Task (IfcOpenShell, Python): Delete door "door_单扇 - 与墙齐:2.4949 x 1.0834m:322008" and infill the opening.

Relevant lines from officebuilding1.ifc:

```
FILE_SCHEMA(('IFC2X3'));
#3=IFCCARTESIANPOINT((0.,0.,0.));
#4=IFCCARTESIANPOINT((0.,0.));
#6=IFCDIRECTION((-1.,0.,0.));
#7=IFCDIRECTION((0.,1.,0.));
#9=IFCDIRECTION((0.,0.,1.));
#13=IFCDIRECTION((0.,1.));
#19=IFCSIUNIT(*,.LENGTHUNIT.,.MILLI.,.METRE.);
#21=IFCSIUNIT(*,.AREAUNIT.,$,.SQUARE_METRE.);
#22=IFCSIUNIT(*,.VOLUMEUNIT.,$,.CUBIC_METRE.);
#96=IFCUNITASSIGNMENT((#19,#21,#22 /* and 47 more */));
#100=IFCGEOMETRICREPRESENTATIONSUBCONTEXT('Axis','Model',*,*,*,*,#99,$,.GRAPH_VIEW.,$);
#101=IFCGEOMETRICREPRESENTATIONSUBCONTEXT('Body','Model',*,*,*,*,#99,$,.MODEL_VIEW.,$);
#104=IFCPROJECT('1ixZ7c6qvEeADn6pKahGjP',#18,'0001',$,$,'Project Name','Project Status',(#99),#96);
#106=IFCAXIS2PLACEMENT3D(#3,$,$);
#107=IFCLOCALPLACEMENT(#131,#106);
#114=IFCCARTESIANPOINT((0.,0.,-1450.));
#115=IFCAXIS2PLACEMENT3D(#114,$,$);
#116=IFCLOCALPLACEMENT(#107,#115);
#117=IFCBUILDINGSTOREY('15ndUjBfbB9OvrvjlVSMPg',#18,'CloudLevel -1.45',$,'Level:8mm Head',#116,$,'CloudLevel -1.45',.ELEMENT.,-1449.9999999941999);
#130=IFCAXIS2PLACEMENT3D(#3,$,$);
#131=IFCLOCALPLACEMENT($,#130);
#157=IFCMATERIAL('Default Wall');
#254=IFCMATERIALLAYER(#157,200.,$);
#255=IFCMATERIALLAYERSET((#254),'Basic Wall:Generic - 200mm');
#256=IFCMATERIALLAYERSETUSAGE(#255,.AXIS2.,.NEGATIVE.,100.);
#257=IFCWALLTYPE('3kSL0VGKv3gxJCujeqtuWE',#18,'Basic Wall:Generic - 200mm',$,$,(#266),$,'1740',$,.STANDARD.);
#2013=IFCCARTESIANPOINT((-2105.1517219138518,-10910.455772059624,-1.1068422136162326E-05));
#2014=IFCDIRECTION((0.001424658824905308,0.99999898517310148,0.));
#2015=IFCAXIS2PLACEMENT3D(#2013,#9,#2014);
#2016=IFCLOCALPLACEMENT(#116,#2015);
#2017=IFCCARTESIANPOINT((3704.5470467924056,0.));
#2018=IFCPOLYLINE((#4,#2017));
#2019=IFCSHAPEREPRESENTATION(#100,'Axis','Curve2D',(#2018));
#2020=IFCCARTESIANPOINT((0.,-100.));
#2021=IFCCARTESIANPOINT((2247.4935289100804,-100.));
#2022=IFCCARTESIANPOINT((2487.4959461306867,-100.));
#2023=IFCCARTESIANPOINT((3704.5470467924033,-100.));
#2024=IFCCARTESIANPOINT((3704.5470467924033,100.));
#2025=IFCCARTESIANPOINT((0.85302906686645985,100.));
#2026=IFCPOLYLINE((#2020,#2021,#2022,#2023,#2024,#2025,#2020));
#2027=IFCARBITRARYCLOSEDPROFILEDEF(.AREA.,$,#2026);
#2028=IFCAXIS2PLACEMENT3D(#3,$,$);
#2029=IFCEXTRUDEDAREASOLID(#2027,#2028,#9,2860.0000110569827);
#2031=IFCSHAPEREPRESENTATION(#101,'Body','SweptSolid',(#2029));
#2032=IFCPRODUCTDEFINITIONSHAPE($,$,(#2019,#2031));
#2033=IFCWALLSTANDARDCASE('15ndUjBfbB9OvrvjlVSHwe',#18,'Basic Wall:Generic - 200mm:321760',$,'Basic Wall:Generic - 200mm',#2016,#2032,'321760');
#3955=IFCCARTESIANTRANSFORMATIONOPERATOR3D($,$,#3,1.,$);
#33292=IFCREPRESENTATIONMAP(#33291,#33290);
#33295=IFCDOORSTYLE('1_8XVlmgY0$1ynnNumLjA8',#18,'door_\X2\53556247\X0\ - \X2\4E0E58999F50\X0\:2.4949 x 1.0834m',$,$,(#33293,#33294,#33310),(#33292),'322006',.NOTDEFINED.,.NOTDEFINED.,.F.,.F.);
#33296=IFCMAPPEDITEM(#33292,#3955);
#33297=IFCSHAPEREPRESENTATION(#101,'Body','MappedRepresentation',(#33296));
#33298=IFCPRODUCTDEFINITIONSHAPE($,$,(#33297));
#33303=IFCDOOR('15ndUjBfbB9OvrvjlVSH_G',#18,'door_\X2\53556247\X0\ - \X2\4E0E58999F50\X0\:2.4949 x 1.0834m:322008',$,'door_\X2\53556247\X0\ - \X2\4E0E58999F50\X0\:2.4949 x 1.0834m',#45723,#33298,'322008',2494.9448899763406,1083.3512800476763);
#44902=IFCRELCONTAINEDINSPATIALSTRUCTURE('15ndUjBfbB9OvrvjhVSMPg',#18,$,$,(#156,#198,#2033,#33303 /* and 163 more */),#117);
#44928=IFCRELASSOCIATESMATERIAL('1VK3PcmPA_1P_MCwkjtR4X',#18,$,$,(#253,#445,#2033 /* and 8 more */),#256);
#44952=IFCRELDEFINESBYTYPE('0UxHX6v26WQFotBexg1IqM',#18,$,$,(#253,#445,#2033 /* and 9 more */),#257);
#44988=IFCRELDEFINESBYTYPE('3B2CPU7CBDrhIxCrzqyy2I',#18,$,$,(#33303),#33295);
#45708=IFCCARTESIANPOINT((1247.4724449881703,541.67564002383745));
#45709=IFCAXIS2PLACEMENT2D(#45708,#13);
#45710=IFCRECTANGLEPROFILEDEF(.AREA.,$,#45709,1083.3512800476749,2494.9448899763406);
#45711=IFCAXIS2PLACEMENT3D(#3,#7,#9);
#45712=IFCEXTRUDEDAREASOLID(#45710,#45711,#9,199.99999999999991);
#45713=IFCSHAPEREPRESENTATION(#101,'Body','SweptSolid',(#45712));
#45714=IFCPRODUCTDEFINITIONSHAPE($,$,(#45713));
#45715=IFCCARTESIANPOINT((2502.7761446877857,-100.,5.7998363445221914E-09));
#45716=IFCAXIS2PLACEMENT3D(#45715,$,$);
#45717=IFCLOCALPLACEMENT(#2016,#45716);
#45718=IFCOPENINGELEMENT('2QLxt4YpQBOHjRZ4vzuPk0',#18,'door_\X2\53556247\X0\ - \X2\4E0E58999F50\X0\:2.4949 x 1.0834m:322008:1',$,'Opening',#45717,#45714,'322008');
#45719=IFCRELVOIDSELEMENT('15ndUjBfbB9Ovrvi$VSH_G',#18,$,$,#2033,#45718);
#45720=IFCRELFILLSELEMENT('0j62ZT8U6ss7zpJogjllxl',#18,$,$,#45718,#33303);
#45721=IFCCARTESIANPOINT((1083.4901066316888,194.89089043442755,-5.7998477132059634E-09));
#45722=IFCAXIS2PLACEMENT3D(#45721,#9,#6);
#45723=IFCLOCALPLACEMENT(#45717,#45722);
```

```python
import ifcopenshell
import ifcopenshell.api.feature
import ifcopenshell.api.root
import ifcopenshell.geom
import ifcopenshell.util.shape

model = ifcopenshell.open("officebuilding1.ifc")
settings = ifcopenshell.geom.settings()


def volume(element):
    """Net volume in cubic metres, openings subtracted."""
    shape = ifcopenshell.geom.create_shape(settings, element)
    return ifcopenshell.util.shape.get_volume(shape.geometry)


door = model.by_guid("15ndUjBfbB9OvrvjlVSH_G")
opening = door.FillsVoids[0].RelatingOpeningElement
wall = opening.VoidsElements[0].RelatingBuildingElement
before = volume(wall)

ifcopenshell.api.root.remove_product(model, product=door)
ifcopenshell.api.feature.remove_feature(model, feature=opening)

after = volume(wall)

print(f"wall volume {before:.3f} -> {after:.3f} m3")

model.write("officebuilding1_edited.ifc")
```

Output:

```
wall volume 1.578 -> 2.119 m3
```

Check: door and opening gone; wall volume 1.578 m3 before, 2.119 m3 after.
